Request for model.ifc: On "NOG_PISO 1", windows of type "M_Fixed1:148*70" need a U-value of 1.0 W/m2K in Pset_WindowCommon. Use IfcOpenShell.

First a look at what the model holds.

```python
import ifcopenshell
import ifcopenshell.util.element

model = ifcopenshell.open("model.ifc")
print(model.schema)
storey = next(s for s in model.by_type("IfcBuildingStorey") if s.Name == "NOG_PISO 1")
windows = [e for e in ifcopenshell.util.element.get_decomposition(storey) if e.is_a("IfcWindow")]
seen = {}
for e in windows:
    element_type = ifcopenshell.util.element.get_type(e)
    key = (element_type.Name if element_type != e and element_type else None, ifcopenshell.util.element.get_pset(e, "Pset_WindowCommon", "ThermalTransmittance"))
    seen[key] = seen.get(key, 0) + 1
for (name, value), count in sorted(seen.items(), key=str):
    print(count, "x", name, "|", value)
```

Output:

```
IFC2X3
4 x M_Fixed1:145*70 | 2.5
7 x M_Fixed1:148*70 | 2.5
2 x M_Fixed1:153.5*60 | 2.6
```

```python
import ifcopenshell
import ifcopenshell.api.pset
import ifcopenshell.util.element

model = ifcopenshell.open("model.ifc")

storey = next(s for s in model.by_type("IfcBuildingStorey") if s.Name == "NOG_PISO 1")
windows = [e for e in ifcopenshell.util.element.get_decomposition(storey) if e.is_a("IfcWindow")]

count = 0
for e in windows:
    element_type = ifcopenshell.util.element.get_type(e)
    if element_type in (None, e) or element_type.Name != "M_Fixed1:148*70":
        continue
    # add_pset returns the element's existing set when there is one.
    pset = ifcopenshell.api.pset.add_pset(model, product=e, name="Pset_WindowCommon")
    ifcopenshell.api.pset.edit_pset(model, pset=pset, properties={"ThermalTransmittance": 1.0})
    count += 1

print(count, "windows updated")

model.write("model_rev.ifc")
```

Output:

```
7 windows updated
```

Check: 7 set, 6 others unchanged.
